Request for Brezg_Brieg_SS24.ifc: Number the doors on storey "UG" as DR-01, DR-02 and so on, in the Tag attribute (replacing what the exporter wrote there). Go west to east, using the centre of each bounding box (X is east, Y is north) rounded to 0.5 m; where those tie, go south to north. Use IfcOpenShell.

First a look at what the model holds.

```python
import ifcopenshell
import ifcopenshell.util.element
import ifcopenshell.util.placement

model = ifcopenshell.open("Brezg_Brieg_SS24.ifc")
print(model.schema)
storey = next(s for s in model.by_type("IfcBuildingStorey") if s.Name == "UG")
doors = [e for e in ifcopenshell.util.element.get_decomposition(storey) if e.is_a("IfcDoor")]
for e in sorted(doors, key=lambda e: e.id()):
    origin = ifcopenshell.util.placement.get_local_placement(e.ObjectPlacement)[:3, 3]
    print(e.id(), e.Tag, e.Name, origin.round(2) + 0.0, sep=" | ")
```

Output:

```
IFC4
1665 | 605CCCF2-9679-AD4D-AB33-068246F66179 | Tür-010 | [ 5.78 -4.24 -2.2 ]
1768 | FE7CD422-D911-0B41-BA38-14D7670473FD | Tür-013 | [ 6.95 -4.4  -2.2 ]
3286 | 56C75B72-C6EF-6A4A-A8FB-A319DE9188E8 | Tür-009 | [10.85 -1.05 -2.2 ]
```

```python
import ifcopenshell
import ifcopenshell.geom
import ifcopenshell.util.element
import ifcopenshell.util.shape

model = ifcopenshell.open("Brezg_Brieg_SS24.ifc")
settings = ifcopenshell.geom.settings()
settings.set("use-world-coords", True)


def centre(element):
    shape = ifcopenshell.geom.create_shape(settings, element)
    return ifcopenshell.util.shape.get_bbox_centroid(shape.geometry)


storey = next(s for s in model.by_type("IfcBuildingStorey") if s.Name == "UG")
doors = [e for e in ifcopenshell.util.element.get_decomposition(storey) if e.is_a("IfcDoor")]

# Insertion points can sit at a corner or the storey origin, so sort by the geometry (in metres).
centres = {e: centre(e) for e in doors}
doors.sort(key=lambda e: (round(centres[e][0] / 0.5), centres[e][1]))

for i, e in enumerate(doors, start=1):
    number = f"DR-{i:02d}"
    e.Tag = number
    print(e.id(), number)

model.write("Brezg_Brieg_SS24_v2.ifc")
```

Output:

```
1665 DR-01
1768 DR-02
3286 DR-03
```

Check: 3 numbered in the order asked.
